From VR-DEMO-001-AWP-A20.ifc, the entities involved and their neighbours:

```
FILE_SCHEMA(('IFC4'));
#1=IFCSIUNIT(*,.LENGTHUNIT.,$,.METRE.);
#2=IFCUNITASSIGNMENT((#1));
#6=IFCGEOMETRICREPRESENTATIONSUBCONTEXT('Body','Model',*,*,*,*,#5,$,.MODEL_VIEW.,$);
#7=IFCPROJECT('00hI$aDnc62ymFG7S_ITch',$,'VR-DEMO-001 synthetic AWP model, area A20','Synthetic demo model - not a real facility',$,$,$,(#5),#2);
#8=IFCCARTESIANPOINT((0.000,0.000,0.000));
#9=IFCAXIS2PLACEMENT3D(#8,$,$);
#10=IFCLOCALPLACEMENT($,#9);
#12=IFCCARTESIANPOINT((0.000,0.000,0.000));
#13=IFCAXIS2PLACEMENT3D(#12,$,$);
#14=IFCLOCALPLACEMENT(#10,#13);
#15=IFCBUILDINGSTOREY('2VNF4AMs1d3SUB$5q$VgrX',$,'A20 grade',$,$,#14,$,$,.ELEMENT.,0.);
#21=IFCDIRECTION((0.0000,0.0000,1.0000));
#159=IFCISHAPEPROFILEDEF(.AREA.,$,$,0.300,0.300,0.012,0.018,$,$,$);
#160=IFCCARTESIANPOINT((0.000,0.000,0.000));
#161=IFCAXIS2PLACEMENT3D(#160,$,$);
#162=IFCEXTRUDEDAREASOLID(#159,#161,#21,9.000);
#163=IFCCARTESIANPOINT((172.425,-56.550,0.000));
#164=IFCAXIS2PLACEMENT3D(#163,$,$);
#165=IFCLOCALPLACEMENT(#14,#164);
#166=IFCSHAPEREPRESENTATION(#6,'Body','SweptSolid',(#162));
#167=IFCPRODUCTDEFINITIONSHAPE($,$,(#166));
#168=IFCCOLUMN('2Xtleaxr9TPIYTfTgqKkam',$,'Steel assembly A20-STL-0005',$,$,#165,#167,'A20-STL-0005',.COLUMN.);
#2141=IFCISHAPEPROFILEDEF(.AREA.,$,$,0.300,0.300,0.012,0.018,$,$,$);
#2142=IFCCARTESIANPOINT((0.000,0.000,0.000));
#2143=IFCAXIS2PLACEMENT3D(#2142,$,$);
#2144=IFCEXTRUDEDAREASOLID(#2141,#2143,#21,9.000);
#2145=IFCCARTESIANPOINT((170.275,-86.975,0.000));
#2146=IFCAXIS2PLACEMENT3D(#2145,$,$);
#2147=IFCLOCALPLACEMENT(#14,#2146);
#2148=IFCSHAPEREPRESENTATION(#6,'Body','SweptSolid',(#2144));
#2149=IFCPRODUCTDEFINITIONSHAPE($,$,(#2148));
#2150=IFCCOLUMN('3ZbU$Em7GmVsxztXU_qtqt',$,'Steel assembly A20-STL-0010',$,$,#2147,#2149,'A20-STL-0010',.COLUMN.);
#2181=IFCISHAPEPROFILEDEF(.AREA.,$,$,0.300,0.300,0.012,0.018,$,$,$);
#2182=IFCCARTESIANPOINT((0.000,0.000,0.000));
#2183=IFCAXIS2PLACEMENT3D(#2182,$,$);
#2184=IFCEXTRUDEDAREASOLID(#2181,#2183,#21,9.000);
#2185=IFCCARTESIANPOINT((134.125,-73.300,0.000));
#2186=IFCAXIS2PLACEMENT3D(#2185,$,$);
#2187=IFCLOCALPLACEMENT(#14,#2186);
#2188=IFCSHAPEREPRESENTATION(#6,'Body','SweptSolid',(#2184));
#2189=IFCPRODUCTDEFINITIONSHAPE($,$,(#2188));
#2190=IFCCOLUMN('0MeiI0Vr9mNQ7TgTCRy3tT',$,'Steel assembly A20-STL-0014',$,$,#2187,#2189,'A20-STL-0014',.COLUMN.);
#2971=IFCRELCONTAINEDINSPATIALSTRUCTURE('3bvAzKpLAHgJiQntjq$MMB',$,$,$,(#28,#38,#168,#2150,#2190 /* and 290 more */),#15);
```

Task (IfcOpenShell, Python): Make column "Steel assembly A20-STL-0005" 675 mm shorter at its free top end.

```python
import ifcopenshell
import ifcopenshell.util.representation
import ifcopenshell.util.unit

model = ifcopenshell.open("VR-DEMO-001-AWP-A20.ifc")
unit_scale = ifcopenshell.util.unit.calculate_unit_scale(model)

member = model.by_id(168)
change = -0.675 / unit_scale

# The extrusion runs towards the end named, so only its depth changes.
body = ifcopenshell.util.representation.get_representation(member, "Model", "Body")
solid = body.Items[0]
old_length = solid.Depth
solid.Depth += change

print(f"length {old_length:g} -> {solid.Depth:g}")

model.write("VR-DEMO-001-AWP-A20-out.ifc")
```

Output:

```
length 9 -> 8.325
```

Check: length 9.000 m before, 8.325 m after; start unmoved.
